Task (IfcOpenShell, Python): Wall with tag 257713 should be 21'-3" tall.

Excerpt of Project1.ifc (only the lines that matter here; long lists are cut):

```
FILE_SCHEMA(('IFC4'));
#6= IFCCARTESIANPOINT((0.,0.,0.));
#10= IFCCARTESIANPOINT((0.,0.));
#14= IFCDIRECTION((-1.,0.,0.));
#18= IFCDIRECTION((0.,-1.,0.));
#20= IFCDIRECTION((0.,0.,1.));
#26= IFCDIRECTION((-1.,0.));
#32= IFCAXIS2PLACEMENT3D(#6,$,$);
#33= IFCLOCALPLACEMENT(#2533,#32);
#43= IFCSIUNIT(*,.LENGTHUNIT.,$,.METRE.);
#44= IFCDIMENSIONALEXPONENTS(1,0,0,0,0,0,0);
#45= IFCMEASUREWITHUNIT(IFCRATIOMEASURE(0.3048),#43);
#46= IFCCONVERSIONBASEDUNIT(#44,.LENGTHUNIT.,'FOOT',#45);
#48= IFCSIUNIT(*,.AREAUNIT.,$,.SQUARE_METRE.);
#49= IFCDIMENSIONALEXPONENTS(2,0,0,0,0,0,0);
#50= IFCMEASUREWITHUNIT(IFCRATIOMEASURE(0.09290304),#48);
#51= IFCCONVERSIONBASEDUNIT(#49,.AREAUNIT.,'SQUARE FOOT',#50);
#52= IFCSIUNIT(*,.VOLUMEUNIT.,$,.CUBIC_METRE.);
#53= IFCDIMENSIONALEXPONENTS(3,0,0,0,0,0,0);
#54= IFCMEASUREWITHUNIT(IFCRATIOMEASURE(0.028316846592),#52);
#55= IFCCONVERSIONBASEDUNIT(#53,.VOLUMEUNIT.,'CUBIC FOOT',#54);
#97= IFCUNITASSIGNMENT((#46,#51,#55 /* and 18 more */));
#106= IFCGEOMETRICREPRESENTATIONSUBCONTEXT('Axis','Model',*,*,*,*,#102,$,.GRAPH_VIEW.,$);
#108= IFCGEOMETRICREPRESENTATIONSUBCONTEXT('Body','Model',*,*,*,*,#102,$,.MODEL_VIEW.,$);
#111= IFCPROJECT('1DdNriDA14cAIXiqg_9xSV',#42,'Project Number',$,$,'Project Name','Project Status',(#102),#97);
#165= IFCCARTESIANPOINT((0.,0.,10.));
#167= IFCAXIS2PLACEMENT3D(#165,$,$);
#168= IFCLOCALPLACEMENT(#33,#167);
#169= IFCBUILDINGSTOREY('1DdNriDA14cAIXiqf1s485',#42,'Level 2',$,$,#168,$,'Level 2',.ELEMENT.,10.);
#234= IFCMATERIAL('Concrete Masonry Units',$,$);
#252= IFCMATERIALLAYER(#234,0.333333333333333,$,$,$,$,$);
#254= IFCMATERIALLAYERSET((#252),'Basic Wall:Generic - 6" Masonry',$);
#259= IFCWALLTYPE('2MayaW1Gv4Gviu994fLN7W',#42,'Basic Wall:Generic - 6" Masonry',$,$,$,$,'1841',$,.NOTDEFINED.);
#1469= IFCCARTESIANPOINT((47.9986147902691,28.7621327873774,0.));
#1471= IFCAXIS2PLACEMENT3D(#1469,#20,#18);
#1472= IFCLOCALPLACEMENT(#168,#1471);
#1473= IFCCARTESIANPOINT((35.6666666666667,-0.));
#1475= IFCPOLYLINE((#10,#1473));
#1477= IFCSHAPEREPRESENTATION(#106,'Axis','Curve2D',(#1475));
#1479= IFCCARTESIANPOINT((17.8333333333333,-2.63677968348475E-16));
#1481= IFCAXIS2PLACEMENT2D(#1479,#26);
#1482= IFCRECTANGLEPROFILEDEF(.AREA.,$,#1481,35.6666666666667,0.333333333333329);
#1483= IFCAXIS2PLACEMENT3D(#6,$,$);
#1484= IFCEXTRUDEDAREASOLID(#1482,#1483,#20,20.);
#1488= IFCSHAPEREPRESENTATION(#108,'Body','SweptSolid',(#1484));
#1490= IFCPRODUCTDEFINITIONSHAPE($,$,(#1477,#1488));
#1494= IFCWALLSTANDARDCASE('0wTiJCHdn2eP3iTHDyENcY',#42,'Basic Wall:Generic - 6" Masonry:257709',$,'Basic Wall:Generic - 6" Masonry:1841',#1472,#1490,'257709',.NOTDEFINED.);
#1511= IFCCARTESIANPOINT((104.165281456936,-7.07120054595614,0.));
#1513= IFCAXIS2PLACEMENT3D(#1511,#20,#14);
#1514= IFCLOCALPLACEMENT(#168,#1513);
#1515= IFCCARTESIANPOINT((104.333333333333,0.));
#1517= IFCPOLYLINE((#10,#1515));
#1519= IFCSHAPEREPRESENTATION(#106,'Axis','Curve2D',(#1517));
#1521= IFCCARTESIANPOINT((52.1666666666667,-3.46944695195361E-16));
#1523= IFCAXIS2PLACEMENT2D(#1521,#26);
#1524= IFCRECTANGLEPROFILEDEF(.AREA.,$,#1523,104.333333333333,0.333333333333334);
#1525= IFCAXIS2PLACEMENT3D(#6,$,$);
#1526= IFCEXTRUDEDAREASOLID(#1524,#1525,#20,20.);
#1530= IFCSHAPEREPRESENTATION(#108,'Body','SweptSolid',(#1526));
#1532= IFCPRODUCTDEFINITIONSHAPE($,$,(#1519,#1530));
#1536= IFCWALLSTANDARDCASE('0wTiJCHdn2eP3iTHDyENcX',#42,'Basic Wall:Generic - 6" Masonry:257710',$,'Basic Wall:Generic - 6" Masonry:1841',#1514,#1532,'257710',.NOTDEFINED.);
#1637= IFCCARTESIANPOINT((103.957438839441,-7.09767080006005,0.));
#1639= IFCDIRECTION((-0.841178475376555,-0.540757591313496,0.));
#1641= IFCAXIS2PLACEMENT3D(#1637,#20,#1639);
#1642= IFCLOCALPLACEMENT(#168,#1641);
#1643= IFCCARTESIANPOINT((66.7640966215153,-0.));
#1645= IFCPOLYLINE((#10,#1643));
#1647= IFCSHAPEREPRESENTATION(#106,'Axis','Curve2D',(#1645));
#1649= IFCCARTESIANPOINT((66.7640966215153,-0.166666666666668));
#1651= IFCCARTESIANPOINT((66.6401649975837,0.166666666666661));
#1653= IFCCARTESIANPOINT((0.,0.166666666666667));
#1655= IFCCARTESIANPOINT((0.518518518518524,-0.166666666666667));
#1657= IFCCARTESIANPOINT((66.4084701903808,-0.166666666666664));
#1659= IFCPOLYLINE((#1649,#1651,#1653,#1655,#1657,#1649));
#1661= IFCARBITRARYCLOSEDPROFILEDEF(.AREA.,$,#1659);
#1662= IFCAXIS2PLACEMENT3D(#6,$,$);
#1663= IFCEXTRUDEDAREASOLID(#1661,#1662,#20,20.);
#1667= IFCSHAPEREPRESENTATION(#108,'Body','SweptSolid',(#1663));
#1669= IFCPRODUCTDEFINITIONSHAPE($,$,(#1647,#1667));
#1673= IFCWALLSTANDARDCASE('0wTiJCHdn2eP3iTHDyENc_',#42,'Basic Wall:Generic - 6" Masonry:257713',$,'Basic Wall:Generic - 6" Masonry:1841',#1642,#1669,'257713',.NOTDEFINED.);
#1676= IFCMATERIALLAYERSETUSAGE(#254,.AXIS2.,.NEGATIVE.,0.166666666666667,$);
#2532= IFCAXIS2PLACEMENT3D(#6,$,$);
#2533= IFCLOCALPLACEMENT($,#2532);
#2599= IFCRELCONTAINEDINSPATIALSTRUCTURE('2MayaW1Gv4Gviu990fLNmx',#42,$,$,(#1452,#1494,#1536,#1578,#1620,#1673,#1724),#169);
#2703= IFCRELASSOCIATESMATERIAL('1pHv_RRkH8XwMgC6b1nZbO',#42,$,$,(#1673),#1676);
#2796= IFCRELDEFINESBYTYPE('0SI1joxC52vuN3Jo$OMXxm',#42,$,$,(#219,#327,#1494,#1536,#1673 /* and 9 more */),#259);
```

```python
import ifcopenshell
import ifcopenshell.geom
import ifcopenshell.util.representation
import ifcopenshell.util.shape
import ifcopenshell.util.unit

model = ifcopenshell.open("Project1.ifc")
unit_scale = ifcopenshell.util.unit.calculate_unit_scale(model)
settings = ifcopenshell.geom.settings()


def volume(element):
    """Net volume in cubic metres, openings subtracted."""
    shape = ifcopenshell.geom.create_shape(settings, element)
    return ifcopenshell.util.shape.get_volume(shape.geometry)


wall = model.by_guid("0wTiJCHdn2eP3iTHDyENc_")
before = volume(wall)

body = ifcopenshell.util.representation.get_representation(wall, "Model", "Body")
solid = body.Items[0]
old_height = solid.Depth
solid.Depth = 255 * 0.0254 / unit_scale
after = volume(wall)

print(f"height {old_height:g} -> {solid.Depth:g}, volume {before:.3f} -> {after:.3f} m3")

model.write("Project1_v2.ifc")
```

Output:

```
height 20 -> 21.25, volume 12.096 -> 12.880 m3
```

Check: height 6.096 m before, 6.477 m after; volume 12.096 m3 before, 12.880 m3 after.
